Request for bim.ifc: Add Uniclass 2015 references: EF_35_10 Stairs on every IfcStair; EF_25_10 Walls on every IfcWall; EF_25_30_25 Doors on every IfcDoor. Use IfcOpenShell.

First a look at what the model holds.

```python
import ifcopenshell

model = ifcopenshell.open("bim.ifc")
print(model.schema)
print("classifications:", [c.Name for c in model.by_type("IfcClassification")])
for ifc_class in ("IfcDoor", "IfcRoof", "IfcStair", "IfcWall", "IfcWindow"):
    print(ifc_class, len(model.by_type(ifc_class)))
```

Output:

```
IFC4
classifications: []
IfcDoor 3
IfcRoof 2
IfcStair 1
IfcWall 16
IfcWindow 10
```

```python
import ifcopenshell
import ifcopenshell.api.classification

model = ifcopenshell.open("bim.ifc")

system = ifcopenshell.api.classification.add_classification(model, classification="Uniclass 2015")

codes = {
    "IfcStair": ("EF_35_10", "Stairs"),
    "IfcWall": ("EF_25_10", "Walls"),
    "IfcDoor": ("EF_25_30_25", "Doors"),
}
for ifc_class, (code, name) in codes.items():
    products = model.by_type(ifc_class)
    ifcopenshell.api.classification.add_reference(
        model, products=products, classification=system, identification=code, name=name
    )
    print(code, len(products))

model.write("bim-out.ifc")
```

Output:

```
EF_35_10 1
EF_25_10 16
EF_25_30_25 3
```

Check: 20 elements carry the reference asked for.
